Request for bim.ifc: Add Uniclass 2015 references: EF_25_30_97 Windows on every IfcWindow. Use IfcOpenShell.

First a look at what the model holds.

```python
import ifcopenshell

model = ifcopenshell.open("bim.ifc")
print(model.schema)
print("classifications:", [c.Name for c in model.by_type("IfcClassification")])
for ifc_class in ("IfcDoor", "IfcRoof", "IfcStair", "IfcWall", "IfcWindow"):
    print(ifc_class, len(model.by_type(ifc_class)))
```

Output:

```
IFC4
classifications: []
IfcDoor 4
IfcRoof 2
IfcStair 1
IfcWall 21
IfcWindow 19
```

```python
import ifcopenshell
import ifcopenshell.api.classification

model = ifcopenshell.open("bim.ifc")

system = ifcopenshell.api.classification.add_classification(model, classification="Uniclass 2015")

codes = {
    "IfcWindow": ("EF_25_30_97", "Windows"),
}
for ifc_class, (code, name) in codes.items():
    products = model.by_type(ifc_class)
    ifcopenshell.api.classification.add_reference(
        model, products=products, classification=system, identification=code, name=name
    )
    print(code, len(products))

model.write("bim_rev.ifc")
```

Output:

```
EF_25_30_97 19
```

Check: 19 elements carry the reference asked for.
